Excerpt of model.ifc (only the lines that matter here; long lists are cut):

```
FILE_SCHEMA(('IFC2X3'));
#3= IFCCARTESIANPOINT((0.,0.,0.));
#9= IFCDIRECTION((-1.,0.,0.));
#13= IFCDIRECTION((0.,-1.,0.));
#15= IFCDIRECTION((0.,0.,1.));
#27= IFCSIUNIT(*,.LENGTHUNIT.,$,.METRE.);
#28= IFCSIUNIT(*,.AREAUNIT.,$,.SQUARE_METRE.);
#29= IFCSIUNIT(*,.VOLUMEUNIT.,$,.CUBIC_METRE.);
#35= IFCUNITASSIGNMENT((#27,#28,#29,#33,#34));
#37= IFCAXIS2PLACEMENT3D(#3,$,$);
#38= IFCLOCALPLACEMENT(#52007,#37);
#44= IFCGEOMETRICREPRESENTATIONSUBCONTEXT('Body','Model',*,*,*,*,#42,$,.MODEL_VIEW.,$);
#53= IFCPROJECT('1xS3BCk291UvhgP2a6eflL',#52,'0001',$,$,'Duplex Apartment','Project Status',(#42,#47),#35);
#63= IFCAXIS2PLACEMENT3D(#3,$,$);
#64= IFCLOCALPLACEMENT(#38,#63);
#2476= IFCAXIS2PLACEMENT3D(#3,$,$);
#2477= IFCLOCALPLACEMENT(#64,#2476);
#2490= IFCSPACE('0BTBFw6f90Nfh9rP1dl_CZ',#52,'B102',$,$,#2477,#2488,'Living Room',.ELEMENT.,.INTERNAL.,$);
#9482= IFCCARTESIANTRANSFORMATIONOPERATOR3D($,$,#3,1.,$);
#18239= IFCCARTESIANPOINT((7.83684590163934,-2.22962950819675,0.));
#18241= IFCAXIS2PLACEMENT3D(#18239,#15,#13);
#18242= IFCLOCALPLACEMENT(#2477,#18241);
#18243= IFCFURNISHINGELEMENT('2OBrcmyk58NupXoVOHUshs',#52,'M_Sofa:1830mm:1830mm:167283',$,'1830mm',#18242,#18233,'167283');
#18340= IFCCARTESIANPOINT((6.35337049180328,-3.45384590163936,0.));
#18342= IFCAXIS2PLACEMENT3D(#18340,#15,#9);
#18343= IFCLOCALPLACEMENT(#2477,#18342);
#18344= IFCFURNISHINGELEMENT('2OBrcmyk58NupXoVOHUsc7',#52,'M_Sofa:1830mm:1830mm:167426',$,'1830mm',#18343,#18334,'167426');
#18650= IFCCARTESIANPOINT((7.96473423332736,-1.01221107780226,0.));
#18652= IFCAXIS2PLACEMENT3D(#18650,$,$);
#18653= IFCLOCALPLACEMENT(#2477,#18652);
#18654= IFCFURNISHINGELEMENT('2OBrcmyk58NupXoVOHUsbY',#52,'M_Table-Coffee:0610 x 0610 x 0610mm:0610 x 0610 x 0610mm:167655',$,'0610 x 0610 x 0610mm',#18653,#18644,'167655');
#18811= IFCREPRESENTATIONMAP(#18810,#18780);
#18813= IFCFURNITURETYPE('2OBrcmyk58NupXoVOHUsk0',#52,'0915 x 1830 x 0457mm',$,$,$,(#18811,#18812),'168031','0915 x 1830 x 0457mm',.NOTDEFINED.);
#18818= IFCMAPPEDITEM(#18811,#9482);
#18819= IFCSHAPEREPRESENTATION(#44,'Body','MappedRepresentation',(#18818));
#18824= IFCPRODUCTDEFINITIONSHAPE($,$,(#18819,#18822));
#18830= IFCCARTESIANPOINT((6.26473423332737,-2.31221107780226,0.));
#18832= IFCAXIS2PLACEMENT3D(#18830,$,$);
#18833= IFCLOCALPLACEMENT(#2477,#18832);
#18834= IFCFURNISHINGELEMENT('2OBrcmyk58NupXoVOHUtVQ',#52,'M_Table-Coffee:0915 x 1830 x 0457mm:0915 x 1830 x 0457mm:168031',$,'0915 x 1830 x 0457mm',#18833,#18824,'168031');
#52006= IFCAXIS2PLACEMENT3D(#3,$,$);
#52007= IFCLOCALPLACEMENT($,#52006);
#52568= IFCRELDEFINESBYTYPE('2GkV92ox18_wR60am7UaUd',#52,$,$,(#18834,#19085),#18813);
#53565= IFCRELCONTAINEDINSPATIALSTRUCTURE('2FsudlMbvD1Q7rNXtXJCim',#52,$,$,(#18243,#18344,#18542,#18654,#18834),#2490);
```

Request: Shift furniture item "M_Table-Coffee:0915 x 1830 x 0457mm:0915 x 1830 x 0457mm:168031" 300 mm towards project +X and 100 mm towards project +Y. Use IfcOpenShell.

```python
import ifcopenshell
import ifcopenshell.api.geometry
import ifcopenshell.util.placement
import ifcopenshell.util.unit

model = ifcopenshell.open("model.ifc")
unit_scale = ifcopenshell.util.unit.calculate_unit_scale(model)

item = model.by_guid("2OBrcmyk58NupXoVOHUtVQ")
matrix = ifcopenshell.util.placement.get_local_placement(item.ObjectPlacement)
matrix[0, 3] += 0.3 / unit_scale
matrix[1, 3] += 0.1 / unit_scale
ifcopenshell.api.geometry.edit_object_placement(model, product=item, matrix=matrix, is_si=False)

print(ifcopenshell.util.placement.get_local_placement(item.ObjectPlacement).round(3) + 0.0)

model.write("model_updated.ifc")
```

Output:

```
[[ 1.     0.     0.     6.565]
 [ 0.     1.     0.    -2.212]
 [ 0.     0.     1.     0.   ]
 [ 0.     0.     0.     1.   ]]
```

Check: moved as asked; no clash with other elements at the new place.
